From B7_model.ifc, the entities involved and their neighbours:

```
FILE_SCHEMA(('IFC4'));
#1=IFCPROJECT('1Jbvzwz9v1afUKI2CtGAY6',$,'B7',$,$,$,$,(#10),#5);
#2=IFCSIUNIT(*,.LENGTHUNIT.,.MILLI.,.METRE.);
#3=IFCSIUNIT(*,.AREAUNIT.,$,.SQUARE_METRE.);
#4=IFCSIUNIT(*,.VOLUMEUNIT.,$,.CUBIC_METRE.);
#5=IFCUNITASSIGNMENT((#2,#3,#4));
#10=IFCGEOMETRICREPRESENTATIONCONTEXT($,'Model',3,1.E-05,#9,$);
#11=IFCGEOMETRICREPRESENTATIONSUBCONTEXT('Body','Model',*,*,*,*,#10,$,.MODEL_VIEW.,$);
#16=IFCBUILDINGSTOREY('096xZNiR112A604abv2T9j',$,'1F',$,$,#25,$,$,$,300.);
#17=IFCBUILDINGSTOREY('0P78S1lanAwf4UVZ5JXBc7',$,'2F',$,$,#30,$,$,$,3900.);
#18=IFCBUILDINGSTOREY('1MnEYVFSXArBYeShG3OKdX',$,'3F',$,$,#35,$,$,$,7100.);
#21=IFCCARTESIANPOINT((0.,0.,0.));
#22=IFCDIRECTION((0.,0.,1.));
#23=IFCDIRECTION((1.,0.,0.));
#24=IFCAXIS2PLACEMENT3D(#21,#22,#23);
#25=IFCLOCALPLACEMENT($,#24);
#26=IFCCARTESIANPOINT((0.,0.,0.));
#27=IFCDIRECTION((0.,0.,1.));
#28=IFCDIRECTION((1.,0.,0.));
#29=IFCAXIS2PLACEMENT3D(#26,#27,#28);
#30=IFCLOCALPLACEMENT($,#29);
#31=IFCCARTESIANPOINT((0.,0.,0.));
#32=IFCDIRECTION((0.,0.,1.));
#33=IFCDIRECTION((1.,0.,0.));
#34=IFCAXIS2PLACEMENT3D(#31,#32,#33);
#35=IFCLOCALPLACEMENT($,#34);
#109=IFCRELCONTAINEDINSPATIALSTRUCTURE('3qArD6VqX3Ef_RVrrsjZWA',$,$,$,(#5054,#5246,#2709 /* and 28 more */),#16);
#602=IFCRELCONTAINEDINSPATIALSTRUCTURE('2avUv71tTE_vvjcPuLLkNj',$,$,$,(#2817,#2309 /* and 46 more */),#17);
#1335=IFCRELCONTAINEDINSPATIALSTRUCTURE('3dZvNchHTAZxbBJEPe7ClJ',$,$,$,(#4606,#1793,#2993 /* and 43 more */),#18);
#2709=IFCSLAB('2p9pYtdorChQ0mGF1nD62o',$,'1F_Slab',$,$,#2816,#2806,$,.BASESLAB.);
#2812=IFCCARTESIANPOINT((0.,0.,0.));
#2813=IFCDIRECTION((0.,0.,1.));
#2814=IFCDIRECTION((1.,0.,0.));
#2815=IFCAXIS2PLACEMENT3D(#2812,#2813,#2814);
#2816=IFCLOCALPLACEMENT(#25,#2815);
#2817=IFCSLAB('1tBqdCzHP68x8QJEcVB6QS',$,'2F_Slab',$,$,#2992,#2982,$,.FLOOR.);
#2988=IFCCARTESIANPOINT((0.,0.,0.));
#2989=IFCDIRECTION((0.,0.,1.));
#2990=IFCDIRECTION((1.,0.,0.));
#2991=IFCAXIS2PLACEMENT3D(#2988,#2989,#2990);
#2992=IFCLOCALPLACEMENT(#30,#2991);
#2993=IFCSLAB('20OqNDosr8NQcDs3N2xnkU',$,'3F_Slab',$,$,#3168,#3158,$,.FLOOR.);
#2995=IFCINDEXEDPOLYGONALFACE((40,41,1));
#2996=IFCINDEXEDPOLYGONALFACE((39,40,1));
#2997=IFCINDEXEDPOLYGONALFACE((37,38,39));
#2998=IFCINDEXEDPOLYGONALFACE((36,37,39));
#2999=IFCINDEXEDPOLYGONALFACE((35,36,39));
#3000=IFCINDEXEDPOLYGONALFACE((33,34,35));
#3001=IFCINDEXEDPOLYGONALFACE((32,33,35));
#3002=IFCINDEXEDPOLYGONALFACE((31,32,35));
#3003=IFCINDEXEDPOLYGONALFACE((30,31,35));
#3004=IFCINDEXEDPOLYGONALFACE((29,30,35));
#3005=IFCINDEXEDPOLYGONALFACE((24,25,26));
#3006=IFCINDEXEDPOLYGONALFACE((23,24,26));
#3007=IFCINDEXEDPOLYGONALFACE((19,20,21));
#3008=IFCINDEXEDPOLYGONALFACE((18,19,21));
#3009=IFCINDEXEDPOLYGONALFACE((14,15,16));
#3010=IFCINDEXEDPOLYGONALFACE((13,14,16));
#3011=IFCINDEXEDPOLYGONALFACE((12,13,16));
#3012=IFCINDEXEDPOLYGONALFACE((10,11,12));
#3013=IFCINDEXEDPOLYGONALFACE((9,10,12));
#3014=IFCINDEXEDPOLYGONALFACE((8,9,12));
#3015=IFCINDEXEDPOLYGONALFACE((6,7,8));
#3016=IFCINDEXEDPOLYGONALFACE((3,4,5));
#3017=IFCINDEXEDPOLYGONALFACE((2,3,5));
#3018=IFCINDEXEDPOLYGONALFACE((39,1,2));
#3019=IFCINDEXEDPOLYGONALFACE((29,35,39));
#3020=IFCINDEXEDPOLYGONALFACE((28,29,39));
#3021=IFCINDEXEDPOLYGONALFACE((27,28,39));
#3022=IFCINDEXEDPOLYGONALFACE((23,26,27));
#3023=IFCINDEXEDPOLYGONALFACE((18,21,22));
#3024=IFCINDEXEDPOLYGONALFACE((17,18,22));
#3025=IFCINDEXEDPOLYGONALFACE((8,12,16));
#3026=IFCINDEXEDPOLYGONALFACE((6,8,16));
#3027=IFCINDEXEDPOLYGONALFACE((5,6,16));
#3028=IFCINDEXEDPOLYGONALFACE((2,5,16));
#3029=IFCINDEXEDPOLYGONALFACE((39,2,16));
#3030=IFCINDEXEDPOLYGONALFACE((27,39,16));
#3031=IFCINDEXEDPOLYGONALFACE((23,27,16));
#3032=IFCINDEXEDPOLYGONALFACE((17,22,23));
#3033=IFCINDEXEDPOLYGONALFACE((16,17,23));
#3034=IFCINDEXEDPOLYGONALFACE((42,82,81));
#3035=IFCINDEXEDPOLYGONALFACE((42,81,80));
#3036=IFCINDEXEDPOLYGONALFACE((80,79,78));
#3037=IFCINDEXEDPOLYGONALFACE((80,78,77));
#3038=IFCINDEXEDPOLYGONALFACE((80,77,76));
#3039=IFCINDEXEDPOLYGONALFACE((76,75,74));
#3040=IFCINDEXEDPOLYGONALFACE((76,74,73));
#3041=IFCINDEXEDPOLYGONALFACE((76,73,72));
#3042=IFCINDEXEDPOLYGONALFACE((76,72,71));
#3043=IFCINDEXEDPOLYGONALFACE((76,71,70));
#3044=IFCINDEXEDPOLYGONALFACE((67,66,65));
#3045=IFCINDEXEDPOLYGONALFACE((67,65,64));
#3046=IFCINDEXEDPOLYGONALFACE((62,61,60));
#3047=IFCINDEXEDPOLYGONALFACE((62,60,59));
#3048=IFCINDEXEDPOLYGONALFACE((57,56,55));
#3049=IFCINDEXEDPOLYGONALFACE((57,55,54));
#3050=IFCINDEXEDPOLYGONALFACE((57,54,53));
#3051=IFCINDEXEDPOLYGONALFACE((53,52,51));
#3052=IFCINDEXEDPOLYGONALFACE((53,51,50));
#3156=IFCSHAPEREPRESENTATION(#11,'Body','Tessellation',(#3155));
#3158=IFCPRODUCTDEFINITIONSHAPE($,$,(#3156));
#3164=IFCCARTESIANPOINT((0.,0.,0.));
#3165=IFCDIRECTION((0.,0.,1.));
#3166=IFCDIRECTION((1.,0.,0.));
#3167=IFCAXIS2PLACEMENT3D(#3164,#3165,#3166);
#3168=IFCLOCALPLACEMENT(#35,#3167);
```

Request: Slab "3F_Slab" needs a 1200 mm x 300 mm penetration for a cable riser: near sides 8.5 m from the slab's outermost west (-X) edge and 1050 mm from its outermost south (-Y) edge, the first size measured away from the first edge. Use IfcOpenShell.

```python
import numpy as np
import ifcopenshell
import ifcopenshell.api.feature
import ifcopenshell.api.geometry
import ifcopenshell.api.root
import ifcopenshell.geom
import ifcopenshell.util.placement
import ifcopenshell.util.representation
import ifcopenshell.util.shape
import ifcopenshell.util.unit

model = ifcopenshell.open("B7_model.ifc")
unit_scale = ifcopenshell.util.unit.calculate_unit_scale(model)
settings = ifcopenshell.geom.settings()


def volume(element):
    """Net volume in cubic metres, openings subtracted."""
    shape = ifcopenshell.geom.create_shape(settings, element)
    return ifcopenshell.util.shape.get_volume(shape.geometry)


slab = model.by_guid("20OqNDosr8NQcDs3N2xnkU")
before = volume(slab)

# Extent in the slab's own axes, in metres. The edges named are its -X and -Y sides.
slab_shape = ifcopenshell.geom.create_shape(settings, slab)
vertices = ifcopenshell.util.shape.get_vertices(slab_shape.geometry)
x_min, y_min, bottom = vertices.min(axis=0)
top = vertices[:, 2].max()

opening = ifcopenshell.api.root.create_entity(model, ifc_class="IfcOpeningElement", name="Cable riser opening", predefined_type="OPENING")
context = ifcopenshell.util.representation.get_context(model, "Model", "Body", "MODEL_VIEW")
width, depth = 1.2, 0.3
outline = [(0.0, 0.0), (width, 0.0), (width, depth), (0.0, depth), (0.0, 0.0)]
# Overshoot both faces by 50 mm so the cut is clean.
shape = ifcopenshell.api.geometry.add_slab_representation(
    model, context=context, depth=top - bottom + 0.1, polyline=outline
)
ifcopenshell.api.geometry.assign_representation(model, product=opening, representation=shape)

matrix = ifcopenshell.util.placement.get_local_placement(slab.ObjectPlacement)
matrix[:, 3] = matrix @ np.append(np.array([x_min + 8.5, y_min + 1.05, bottom - 0.05]) / unit_scale, 1.0)
ifcopenshell.api.geometry.edit_object_placement(model, product=opening, matrix=matrix, is_si=False)
ifcopenshell.api.feature.add_feature(model, feature=opening, element=slab)

after = volume(slab)

print(f"slab volume {before:.3f} -> {after:.3f} m3")

model.write("B7_model-out.ifc")
```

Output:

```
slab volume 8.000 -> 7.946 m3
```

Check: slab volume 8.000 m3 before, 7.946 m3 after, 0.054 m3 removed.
